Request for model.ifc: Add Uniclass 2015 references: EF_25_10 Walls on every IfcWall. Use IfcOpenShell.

First a look at what the model holds.

```python
import ifcopenshell

model = ifcopenshell.open("model.ifc")
print(model.schema)
print("classifications:", [c.Name for c in model.by_type("IfcClassification")])
for ifc_class in ("IfcDoor", "IfcRoof", "IfcStair", "IfcWall", "IfcWindow"):
    print(ifc_class, len(model.by_type(ifc_class)))
```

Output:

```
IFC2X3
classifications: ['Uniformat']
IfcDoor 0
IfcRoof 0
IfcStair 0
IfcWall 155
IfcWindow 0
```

```python
import ifcopenshell
import ifcopenshell.api.classification

model = ifcopenshell.open("model.ifc")

# IFC2X3 requires Source and Edition and has no link from the project to the system.
system = model.create_entity("IfcClassification", Source="NBS", Edition="2015", Name="Uniclass 2015")

codes = {
    "IfcWall": ("EF_25_10", "Walls"),
}
for ifc_class, (code, name) in codes.items():
    products = model.by_type(ifc_class)
    ifcopenshell.api.classification.add_reference(
        model, products=products, classification=system, identification=code, name=name
    )
    print(code, len(products))

model.write("model_updated.ifc")
```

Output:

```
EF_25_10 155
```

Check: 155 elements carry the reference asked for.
